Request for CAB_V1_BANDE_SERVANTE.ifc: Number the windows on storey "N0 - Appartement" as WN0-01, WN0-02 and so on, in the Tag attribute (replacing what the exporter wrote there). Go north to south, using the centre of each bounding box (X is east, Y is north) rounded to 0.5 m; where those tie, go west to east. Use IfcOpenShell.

First a look at what the model holds.

```python
import ifcopenshell
import ifcopenshell.util.element
import ifcopenshell.util.placement

model = ifcopenshell.open("CAB_V1_BANDE_SERVANTE.ifc")
print(model.schema)
storey = next(s for s in model.by_type("IfcBuildingStorey") if s.Name == "N0 - Appartement")
windows = [e for e in ifcopenshell.util.element.get_decomposition(storey) if e.is_a("IfcWindow")]
for e in sorted(windows, key=lambda e: e.id()):
    origin = ifcopenshell.util.placement.get_local_placement(e.ObjectPlacement)[:3, 3]
    print(e.id(), e.Tag, e.Name, origin.round(2) + 0.0, sep=" | ")
```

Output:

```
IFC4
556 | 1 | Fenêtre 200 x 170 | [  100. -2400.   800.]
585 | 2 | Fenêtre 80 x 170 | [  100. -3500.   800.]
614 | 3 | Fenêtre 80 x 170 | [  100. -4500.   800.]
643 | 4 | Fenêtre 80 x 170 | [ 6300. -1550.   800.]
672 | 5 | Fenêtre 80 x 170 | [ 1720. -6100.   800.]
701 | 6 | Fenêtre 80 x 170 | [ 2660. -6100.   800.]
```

```python
import ifcopenshell
import ifcopenshell.geom
import ifcopenshell.util.element
import ifcopenshell.util.shape

model = ifcopenshell.open("CAB_V1_BANDE_SERVANTE.ifc")
settings = ifcopenshell.geom.settings()
settings.set("use-world-coords", True)


def centre(element):
    shape = ifcopenshell.geom.create_shape(settings, element)
    return ifcopenshell.util.shape.get_bbox_centroid(shape.geometry)


storey = next(s for s in model.by_type("IfcBuildingStorey") if s.Name == "N0 - Appartement")
windows = [e for e in ifcopenshell.util.element.get_decomposition(storey) if e.is_a("IfcWindow")]

# Insertion points can sit at a corner or the storey origin, so sort by the geometry (in metres).
centres = {e: centre(e) for e in windows}
windows.sort(key=lambda e: (-round(centres[e][1] / 0.5), centres[e][0]))

for i, e in enumerate(windows, start=1):
    number = f"WN0-{i:02d}"
    e.Tag = number
    print(e.id(), number)

model.write("CAB_V1_BANDE_SERVANTE_edited.ifc")
```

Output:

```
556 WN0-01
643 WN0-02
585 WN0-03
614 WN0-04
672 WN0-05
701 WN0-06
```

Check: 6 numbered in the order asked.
